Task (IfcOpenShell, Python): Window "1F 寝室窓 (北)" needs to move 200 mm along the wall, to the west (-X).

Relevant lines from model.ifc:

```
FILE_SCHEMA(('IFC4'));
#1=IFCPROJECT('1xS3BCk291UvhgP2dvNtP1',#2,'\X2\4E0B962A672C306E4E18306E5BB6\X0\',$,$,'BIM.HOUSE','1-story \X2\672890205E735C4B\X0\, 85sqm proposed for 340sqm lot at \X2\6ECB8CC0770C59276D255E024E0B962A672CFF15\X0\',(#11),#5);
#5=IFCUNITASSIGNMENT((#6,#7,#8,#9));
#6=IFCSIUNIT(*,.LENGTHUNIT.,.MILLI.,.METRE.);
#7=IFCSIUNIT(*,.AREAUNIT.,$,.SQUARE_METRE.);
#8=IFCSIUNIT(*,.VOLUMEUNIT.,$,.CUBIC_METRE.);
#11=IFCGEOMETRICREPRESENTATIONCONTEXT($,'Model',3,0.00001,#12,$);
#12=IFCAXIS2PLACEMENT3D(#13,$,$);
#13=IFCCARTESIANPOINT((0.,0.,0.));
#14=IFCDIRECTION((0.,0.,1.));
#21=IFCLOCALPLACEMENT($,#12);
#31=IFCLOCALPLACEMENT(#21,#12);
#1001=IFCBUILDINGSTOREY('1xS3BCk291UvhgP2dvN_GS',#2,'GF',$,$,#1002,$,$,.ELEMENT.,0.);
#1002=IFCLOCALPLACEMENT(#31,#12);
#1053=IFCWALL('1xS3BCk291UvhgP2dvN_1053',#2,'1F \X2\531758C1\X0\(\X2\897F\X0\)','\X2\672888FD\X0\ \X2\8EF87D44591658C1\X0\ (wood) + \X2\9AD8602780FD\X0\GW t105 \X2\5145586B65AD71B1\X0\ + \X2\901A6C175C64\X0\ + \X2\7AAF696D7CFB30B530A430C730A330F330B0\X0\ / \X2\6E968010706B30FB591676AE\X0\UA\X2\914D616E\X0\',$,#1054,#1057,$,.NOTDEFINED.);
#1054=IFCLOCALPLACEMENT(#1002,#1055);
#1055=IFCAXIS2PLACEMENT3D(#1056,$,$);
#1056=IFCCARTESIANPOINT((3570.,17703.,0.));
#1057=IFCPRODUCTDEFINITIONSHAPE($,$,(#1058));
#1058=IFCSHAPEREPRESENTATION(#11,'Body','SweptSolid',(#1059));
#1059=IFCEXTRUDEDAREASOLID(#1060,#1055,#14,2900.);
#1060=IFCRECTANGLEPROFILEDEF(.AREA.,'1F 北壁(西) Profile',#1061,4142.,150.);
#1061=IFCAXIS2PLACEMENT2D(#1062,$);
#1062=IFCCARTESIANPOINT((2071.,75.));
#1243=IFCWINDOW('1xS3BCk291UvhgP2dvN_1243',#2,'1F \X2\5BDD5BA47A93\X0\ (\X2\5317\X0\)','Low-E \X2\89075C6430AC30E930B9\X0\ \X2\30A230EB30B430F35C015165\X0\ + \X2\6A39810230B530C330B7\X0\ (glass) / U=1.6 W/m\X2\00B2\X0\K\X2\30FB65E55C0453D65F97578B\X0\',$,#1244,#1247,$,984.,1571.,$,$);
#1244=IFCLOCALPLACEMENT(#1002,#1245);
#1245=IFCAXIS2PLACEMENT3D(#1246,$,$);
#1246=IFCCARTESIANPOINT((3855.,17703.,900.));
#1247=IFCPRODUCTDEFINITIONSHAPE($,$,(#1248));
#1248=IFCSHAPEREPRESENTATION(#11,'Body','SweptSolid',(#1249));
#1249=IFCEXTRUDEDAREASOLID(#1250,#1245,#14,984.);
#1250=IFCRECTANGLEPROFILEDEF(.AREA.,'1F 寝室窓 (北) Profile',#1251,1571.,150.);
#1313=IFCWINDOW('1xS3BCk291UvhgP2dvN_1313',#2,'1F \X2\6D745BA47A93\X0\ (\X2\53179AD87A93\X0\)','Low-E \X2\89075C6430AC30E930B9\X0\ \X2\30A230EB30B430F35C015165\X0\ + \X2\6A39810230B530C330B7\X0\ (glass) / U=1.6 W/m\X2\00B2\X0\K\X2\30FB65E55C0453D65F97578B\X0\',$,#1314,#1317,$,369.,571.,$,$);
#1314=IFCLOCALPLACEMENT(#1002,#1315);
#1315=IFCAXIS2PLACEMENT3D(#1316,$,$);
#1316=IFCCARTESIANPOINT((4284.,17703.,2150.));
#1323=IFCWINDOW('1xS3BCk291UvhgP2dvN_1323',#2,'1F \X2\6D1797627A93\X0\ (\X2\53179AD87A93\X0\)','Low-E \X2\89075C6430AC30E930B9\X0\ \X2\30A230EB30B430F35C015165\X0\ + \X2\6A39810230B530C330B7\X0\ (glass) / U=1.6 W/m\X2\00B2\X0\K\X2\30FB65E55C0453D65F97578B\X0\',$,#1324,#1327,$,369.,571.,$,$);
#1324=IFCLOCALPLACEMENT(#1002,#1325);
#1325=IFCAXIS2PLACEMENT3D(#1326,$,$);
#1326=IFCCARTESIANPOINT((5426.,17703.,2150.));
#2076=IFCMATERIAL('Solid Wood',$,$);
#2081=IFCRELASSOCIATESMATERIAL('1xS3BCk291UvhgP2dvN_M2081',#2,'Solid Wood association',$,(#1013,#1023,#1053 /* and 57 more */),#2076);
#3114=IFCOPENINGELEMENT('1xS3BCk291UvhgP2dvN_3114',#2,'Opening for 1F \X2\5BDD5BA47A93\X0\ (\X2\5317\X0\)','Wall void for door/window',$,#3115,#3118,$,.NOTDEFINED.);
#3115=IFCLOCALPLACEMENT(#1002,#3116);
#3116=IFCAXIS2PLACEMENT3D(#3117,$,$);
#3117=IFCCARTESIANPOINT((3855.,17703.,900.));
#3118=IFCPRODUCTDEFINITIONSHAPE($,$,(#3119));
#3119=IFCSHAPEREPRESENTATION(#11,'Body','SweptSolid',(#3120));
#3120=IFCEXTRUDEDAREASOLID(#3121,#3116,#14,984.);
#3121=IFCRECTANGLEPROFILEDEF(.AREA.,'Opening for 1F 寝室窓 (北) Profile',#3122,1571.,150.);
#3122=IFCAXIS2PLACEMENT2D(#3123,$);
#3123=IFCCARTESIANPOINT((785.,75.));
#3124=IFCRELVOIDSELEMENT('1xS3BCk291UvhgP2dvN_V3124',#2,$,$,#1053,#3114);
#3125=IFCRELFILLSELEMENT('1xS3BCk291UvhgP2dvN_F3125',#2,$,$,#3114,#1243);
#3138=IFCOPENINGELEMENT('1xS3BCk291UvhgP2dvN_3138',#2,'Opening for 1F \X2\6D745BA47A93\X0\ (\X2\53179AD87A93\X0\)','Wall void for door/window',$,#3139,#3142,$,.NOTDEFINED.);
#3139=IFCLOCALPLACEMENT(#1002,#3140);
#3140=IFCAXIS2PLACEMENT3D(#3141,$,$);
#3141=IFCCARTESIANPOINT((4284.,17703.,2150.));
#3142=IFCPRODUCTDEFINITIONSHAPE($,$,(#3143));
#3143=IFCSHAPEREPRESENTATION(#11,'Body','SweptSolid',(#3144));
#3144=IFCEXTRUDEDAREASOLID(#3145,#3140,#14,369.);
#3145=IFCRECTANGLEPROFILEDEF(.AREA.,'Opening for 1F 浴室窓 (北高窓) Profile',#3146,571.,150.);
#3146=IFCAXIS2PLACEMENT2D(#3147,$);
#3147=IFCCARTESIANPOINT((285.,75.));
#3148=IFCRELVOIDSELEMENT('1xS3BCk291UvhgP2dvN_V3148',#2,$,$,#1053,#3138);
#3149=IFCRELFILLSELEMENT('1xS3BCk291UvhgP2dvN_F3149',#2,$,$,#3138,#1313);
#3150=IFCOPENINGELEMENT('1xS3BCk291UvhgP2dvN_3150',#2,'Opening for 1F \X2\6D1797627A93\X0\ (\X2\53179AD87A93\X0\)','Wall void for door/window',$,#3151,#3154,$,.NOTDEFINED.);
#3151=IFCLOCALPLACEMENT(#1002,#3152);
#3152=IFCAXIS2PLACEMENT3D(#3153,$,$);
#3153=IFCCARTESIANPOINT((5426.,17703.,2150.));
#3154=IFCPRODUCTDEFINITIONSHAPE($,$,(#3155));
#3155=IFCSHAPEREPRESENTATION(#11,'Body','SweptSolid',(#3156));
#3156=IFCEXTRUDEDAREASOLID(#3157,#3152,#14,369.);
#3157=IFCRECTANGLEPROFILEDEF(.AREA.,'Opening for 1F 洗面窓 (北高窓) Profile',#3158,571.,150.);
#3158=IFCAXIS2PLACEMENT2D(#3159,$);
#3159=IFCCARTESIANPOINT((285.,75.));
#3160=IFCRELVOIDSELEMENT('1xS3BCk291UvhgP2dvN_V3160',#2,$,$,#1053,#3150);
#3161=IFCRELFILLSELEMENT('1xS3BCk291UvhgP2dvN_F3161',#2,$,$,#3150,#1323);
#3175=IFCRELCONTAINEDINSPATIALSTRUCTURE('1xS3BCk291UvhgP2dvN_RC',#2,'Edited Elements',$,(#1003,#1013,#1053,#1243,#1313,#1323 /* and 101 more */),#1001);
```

```python
import ifcopenshell
import ifcopenshell.api.geometry
import ifcopenshell.util.placement
import ifcopenshell.util.unit

model = ifcopenshell.open("model.ifc")
unit_scale = ifcopenshell.util.unit.calculate_unit_scale(model)

window = model.by_guid("1xS3BCk291UvhgP2dvN_1243")
opening = window.FillsVoids[0].RelatingOpeningElement
wall = opening.VoidsElements[0].RelatingBuildingElement

wall_matrix = ifcopenshell.util.placement.get_local_placement(wall.ObjectPlacement)
shift = wall_matrix[:3, 0] * -0.2 / unit_scale
before = ifcopenshell.util.placement.get_local_placement(window.ObjectPlacement)[:3, 3].copy()

# The window is not placed relative to its opening, so move both.
for product in (opening, window):
    matrix = ifcopenshell.util.placement.get_local_placement(product.ObjectPlacement)
    matrix[:3, 3] += shift
    ifcopenshell.api.geometry.edit_object_placement(model, product=product, matrix=matrix, is_si=False)

after = ifcopenshell.util.placement.get_local_placement(window.ObjectPlacement)[:3, 3]
print("window moved by", (after - before).round(3) + 0.0)

model.write("model_rev.ifc")
```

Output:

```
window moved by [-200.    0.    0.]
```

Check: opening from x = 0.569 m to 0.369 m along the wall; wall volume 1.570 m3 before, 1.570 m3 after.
